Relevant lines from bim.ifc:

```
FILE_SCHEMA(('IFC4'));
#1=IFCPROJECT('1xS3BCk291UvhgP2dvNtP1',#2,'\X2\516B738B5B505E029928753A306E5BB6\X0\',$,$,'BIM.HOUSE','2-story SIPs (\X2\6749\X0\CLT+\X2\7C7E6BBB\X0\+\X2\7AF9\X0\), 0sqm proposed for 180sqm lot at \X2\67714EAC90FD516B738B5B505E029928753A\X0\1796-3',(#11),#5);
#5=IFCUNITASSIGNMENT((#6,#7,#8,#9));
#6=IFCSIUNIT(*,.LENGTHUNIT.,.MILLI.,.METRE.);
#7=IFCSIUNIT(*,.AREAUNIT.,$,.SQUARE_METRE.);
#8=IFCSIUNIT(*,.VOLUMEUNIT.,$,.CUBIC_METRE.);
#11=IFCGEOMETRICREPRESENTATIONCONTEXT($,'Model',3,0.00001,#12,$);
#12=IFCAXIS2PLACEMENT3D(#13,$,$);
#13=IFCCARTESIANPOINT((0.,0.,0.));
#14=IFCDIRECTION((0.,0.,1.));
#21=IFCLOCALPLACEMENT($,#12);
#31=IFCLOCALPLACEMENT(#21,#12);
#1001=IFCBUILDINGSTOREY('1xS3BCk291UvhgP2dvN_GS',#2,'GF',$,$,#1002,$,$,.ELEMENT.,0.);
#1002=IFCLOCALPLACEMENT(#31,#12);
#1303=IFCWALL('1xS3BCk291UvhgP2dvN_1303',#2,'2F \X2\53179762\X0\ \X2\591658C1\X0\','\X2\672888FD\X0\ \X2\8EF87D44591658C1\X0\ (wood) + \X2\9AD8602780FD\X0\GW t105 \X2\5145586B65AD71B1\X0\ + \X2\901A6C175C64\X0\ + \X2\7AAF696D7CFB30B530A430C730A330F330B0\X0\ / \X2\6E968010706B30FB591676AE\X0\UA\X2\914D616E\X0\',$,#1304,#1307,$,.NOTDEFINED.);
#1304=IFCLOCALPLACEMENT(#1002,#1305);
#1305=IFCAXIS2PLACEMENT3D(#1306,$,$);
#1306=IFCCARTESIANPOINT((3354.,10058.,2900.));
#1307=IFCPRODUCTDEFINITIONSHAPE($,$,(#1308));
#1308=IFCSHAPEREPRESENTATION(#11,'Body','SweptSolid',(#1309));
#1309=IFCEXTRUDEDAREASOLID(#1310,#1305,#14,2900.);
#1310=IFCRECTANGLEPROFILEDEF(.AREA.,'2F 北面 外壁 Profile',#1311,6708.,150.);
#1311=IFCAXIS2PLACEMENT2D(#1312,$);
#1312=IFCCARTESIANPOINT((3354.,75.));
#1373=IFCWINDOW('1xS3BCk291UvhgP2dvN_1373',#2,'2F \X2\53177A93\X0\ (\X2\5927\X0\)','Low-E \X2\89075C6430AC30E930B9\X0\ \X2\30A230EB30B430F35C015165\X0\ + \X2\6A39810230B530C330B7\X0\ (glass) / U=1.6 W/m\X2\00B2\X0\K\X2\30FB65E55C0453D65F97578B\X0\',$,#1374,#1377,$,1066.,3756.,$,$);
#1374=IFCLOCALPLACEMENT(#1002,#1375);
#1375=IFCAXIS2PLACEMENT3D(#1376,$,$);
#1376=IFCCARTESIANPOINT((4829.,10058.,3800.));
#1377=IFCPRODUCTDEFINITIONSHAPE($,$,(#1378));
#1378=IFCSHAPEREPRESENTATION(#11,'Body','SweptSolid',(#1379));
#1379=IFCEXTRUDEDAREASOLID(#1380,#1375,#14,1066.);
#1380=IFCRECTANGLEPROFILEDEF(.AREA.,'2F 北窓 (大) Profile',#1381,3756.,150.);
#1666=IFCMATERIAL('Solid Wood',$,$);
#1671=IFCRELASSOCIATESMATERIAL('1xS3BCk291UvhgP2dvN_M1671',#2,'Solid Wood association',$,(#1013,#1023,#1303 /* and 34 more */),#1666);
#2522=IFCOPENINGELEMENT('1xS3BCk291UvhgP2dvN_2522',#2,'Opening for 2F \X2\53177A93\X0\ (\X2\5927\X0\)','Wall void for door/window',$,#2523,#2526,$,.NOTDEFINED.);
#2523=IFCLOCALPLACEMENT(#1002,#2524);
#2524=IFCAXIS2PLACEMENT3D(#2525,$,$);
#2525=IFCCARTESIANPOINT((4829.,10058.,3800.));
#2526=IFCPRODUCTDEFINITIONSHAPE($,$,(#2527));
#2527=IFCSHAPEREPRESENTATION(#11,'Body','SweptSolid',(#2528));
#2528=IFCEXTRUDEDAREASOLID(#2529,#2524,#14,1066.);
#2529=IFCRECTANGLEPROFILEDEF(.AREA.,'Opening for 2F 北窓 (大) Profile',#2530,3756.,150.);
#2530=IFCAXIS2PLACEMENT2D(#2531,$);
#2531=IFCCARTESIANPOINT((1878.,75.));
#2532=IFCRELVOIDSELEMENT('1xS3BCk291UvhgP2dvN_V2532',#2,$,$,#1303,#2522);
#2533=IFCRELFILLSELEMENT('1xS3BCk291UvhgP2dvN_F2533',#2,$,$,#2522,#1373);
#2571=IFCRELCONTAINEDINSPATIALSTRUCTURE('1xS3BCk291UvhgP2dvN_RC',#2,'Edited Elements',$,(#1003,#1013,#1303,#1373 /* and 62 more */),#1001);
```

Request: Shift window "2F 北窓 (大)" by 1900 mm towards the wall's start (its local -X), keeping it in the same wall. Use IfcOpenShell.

```python
import ifcopenshell
import ifcopenshell.api.geometry
import ifcopenshell.util.placement
import ifcopenshell.util.unit

model = ifcopenshell.open("bim.ifc")
unit_scale = ifcopenshell.util.unit.calculate_unit_scale(model)

window = model.by_id(1373)
opening = window.FillsVoids[0].RelatingOpeningElement
wall = opening.VoidsElements[0].RelatingBuildingElement

wall_matrix = ifcopenshell.util.placement.get_local_placement(wall.ObjectPlacement)
shift = wall_matrix[:3, 0] * -1.9 / unit_scale
before = ifcopenshell.util.placement.get_local_placement(window.ObjectPlacement)[:3, 3].copy()

# The window is not placed relative to its opening, so move both.
for product in (opening, window):
    matrix = ifcopenshell.util.placement.get_local_placement(product.ObjectPlacement)
    matrix[:3, 3] += shift
    ifcopenshell.api.geometry.edit_object_placement(model, product=product, matrix=matrix, is_si=False)

after = ifcopenshell.util.placement.get_local_placement(window.ObjectPlacement)[:3, 3]
print("window moved by", (after - before).round(3) + 0.0)

model.write("bim_edited.ifc")
```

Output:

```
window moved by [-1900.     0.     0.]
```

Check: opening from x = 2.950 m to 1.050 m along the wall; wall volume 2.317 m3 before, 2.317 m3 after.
